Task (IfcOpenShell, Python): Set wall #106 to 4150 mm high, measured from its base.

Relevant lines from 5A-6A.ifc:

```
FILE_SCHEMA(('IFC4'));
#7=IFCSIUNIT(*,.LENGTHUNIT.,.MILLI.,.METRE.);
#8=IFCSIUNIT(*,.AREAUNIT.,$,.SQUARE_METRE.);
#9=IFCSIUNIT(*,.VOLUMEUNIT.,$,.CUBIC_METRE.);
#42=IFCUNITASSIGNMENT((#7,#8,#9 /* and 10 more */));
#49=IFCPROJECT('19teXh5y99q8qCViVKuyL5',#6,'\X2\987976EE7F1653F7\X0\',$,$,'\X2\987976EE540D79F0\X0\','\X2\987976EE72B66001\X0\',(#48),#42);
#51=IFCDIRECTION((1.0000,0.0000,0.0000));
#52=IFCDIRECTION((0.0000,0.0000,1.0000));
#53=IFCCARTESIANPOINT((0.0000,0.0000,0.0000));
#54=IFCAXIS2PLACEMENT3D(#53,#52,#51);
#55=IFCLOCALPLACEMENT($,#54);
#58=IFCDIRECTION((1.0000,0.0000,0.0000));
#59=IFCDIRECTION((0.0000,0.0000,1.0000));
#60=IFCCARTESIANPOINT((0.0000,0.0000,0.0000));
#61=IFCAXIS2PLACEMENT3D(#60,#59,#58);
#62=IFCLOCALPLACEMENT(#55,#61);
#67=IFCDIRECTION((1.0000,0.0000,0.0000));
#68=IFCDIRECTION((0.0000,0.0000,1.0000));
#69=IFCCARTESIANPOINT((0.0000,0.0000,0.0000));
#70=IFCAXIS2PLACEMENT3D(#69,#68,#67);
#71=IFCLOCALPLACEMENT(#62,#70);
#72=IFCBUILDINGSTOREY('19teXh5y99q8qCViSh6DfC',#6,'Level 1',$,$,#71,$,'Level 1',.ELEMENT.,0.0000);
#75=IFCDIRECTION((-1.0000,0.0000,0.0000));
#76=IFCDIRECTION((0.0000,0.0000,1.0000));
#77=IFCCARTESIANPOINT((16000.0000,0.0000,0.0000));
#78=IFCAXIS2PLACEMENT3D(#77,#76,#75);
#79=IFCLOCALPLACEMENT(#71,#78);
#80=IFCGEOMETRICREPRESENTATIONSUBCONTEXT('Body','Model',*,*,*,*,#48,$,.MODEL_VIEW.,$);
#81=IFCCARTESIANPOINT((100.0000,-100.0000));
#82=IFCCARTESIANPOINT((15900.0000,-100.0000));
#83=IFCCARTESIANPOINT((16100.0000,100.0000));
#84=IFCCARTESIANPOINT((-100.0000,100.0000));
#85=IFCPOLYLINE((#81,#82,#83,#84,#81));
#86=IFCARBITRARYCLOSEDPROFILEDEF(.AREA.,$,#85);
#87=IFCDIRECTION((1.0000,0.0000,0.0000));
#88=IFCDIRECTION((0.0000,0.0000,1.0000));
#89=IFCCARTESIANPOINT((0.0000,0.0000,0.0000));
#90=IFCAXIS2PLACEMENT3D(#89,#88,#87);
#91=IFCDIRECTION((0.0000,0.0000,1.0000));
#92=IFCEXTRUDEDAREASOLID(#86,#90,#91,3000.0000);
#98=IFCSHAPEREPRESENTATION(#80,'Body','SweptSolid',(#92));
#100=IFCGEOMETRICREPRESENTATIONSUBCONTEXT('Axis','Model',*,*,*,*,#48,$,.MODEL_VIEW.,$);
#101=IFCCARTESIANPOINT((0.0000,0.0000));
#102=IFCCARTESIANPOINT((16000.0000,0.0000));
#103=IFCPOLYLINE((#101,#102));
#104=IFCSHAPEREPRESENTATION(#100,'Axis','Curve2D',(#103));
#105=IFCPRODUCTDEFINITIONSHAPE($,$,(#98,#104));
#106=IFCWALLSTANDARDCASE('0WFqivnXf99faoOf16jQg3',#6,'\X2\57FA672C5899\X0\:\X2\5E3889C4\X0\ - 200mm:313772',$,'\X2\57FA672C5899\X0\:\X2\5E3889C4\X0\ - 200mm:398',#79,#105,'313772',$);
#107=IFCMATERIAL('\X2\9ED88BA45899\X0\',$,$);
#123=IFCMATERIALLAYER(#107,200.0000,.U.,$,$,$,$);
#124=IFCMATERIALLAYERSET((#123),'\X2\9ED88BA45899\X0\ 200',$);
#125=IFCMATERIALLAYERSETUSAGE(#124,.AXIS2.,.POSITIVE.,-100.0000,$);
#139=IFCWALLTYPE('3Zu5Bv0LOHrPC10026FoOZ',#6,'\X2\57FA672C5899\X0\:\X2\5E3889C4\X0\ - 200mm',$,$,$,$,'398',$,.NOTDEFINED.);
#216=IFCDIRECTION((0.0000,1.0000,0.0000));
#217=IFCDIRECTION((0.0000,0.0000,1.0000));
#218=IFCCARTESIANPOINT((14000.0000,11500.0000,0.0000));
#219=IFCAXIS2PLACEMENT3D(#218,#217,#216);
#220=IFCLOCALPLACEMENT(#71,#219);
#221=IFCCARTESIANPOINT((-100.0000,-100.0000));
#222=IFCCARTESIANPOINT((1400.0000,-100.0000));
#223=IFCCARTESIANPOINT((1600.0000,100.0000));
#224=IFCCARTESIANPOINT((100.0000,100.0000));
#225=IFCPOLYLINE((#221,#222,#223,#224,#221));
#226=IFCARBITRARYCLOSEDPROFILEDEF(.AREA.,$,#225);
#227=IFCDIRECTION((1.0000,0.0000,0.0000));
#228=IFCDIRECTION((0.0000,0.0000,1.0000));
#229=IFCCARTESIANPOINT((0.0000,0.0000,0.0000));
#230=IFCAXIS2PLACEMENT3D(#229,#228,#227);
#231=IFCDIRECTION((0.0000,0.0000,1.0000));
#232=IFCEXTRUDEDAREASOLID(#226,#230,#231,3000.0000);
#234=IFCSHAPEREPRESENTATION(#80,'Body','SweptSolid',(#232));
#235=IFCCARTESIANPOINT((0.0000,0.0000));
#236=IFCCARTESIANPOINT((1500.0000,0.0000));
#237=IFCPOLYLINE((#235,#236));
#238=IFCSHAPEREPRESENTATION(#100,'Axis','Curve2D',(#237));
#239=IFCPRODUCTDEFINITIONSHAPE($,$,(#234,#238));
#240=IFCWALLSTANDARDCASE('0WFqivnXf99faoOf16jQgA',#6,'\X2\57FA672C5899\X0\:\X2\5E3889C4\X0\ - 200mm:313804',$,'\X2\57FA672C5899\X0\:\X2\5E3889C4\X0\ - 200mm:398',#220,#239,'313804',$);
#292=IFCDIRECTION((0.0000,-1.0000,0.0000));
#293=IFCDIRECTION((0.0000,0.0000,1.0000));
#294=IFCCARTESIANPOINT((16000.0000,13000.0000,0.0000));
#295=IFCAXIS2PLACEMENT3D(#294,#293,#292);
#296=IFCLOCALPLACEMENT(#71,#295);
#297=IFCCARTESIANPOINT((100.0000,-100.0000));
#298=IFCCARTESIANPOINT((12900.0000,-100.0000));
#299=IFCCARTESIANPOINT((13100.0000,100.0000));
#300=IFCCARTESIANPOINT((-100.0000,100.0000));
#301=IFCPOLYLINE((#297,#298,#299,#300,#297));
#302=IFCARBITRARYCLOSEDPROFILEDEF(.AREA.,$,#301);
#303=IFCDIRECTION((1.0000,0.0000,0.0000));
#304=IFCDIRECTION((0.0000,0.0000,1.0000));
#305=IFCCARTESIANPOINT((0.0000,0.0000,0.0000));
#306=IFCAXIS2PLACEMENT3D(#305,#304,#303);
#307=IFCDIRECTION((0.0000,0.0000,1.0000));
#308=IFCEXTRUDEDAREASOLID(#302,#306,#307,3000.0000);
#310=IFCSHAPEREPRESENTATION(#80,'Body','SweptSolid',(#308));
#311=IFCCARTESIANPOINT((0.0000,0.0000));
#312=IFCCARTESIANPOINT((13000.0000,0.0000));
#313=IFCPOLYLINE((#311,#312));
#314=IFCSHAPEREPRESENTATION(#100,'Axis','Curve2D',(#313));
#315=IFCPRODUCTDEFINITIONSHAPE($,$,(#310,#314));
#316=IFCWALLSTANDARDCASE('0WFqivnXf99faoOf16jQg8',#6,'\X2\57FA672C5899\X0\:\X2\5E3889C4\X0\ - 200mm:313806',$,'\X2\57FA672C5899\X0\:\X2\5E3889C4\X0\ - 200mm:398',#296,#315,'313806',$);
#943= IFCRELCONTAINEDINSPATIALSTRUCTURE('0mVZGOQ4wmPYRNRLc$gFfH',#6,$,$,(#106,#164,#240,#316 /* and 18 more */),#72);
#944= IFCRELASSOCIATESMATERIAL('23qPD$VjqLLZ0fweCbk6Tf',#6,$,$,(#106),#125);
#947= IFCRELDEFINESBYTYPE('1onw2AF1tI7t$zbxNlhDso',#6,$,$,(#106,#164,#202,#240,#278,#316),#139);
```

```python
import ifcopenshell
import ifcopenshell.geom
import ifcopenshell.util.representation
import ifcopenshell.util.shape

model = ifcopenshell.open("5A-6A.ifc")
settings = ifcopenshell.geom.settings()


def volume(element):
    """Net volume in cubic metres, openings subtracted."""
    shape = ifcopenshell.geom.create_shape(settings, element)
    return ifcopenshell.util.shape.get_volume(shape.geometry)


wall = model.by_guid("0WFqivnXf99faoOf16jQg3")
before = volume(wall)

body = ifcopenshell.util.representation.get_representation(wall, "Model", "Body")
solid = body.Items[0]
old_height = solid.Depth
solid.Depth = 4150.0
after = volume(wall)

print(f"height {old_height:g} -> {solid.Depth:g}, volume {before:.3f} -> {after:.3f} m3")

model.write("5A-6A_v2.ifc")
```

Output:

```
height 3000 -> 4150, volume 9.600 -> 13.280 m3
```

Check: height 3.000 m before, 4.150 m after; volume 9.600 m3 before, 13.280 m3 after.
